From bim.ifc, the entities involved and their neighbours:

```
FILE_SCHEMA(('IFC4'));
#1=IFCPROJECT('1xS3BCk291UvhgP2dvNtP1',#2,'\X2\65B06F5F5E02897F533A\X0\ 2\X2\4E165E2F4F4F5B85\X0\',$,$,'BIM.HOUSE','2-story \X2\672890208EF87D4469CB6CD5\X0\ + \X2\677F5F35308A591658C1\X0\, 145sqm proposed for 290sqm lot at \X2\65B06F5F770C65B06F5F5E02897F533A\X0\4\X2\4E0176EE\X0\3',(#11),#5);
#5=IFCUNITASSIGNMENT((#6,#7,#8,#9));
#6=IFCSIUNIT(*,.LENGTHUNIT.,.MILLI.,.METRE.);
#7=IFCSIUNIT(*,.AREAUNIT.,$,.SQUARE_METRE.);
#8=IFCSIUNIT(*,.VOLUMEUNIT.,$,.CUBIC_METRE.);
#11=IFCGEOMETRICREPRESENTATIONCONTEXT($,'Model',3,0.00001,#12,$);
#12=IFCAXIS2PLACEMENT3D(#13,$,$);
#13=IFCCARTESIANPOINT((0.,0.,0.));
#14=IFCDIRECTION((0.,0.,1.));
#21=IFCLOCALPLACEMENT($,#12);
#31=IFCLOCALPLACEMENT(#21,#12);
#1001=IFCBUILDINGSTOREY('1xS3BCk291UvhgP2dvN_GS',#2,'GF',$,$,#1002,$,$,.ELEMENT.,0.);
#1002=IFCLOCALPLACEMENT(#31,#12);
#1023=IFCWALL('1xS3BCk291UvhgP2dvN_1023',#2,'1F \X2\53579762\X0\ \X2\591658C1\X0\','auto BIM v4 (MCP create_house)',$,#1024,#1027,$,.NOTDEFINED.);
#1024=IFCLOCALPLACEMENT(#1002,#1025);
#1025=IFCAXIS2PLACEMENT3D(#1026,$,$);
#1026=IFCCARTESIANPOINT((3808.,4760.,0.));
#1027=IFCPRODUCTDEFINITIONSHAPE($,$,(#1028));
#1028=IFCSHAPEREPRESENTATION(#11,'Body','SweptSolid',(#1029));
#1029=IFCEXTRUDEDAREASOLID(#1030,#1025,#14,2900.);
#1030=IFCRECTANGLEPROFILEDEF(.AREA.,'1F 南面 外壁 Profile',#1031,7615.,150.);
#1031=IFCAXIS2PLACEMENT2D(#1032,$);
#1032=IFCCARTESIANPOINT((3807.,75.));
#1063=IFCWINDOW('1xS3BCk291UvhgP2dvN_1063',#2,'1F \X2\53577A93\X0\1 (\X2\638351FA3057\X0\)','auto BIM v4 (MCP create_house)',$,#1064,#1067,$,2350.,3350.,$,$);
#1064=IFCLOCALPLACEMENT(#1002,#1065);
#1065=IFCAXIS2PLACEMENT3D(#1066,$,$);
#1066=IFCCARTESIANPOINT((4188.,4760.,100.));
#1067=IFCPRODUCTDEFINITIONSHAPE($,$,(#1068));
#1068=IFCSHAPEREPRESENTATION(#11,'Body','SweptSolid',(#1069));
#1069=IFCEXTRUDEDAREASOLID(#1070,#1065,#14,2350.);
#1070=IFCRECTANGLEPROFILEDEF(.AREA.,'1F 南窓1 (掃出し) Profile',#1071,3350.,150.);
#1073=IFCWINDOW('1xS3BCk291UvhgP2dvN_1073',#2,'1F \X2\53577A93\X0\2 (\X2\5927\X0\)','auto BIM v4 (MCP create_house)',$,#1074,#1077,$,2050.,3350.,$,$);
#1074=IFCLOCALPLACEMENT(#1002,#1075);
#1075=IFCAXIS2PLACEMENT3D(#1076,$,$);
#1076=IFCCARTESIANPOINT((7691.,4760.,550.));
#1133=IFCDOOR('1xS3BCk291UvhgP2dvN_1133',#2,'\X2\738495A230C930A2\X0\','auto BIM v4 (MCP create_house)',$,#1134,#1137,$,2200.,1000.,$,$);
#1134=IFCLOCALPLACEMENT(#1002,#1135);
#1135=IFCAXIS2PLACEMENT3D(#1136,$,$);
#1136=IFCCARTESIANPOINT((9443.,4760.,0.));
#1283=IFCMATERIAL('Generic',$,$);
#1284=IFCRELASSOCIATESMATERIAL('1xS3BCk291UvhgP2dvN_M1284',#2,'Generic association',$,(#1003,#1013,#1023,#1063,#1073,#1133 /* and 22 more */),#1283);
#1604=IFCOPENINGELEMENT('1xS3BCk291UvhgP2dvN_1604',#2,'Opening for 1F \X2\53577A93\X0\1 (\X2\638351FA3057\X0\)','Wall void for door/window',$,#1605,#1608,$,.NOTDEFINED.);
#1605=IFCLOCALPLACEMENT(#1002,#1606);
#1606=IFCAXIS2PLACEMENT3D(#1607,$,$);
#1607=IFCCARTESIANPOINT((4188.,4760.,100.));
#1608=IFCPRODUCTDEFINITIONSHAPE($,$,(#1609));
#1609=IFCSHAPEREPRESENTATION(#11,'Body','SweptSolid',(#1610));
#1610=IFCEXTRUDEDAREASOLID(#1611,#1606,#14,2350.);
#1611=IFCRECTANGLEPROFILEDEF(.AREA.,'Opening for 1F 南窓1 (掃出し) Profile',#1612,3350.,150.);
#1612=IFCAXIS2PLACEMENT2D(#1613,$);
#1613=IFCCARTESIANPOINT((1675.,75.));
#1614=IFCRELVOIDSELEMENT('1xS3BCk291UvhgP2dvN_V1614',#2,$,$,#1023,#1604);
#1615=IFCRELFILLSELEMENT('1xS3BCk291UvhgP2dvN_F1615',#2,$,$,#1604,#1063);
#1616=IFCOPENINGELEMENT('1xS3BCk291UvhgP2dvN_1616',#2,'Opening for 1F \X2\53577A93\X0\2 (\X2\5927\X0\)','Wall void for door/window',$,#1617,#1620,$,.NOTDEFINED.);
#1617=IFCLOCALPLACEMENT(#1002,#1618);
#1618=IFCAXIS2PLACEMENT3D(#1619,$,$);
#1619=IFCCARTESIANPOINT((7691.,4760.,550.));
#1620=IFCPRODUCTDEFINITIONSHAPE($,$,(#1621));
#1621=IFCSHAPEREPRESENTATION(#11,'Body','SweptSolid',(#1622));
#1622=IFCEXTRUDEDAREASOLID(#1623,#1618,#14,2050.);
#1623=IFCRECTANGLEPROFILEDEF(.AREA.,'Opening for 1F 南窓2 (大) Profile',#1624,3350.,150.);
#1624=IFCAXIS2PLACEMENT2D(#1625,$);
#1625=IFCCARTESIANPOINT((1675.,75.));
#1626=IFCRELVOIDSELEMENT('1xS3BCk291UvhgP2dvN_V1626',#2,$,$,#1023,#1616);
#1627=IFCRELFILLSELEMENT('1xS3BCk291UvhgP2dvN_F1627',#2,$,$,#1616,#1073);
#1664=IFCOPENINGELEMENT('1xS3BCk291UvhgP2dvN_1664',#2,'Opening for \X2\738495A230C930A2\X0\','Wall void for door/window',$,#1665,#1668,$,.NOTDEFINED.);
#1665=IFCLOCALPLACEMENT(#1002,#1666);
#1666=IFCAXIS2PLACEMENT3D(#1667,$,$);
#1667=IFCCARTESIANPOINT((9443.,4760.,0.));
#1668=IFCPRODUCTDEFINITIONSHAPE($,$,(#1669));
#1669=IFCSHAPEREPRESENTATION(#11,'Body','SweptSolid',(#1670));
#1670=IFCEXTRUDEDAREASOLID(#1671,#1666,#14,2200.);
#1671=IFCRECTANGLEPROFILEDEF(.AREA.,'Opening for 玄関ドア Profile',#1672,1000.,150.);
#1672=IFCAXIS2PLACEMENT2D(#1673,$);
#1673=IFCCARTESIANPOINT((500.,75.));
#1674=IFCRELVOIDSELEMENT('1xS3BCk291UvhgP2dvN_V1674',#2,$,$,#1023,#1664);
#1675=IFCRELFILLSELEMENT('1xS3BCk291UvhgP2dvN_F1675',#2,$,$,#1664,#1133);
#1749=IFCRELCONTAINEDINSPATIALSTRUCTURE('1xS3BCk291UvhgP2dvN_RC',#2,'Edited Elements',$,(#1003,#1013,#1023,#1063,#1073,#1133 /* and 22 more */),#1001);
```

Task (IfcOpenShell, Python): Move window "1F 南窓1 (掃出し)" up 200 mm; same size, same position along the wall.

```python
import numpy as np
import ifcopenshell
import ifcopenshell.api.geometry
import ifcopenshell.util.placement
import ifcopenshell.util.unit

model = ifcopenshell.open("bim.ifc")
unit_scale = ifcopenshell.util.unit.calculate_unit_scale(model)

window = model.by_id(1063)
opening = window.FillsVoids[0].RelatingOpeningElement
dz = 200.0

shift = np.array([0.0, 0.0, dz])
# The window is not placed relative to its opening, so move both.
for product in (opening, window):
    matrix = ifcopenshell.util.placement.get_local_placement(product.ObjectPlacement)
    matrix[:3, 3] += shift
    ifcopenshell.api.geometry.edit_object_placement(model, product=product, matrix=matrix, is_si=False)

print(f"moved by {dz * unit_scale:+.3f} m")

model.write("bim-out.ifc")
```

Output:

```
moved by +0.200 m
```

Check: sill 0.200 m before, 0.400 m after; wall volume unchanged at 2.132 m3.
